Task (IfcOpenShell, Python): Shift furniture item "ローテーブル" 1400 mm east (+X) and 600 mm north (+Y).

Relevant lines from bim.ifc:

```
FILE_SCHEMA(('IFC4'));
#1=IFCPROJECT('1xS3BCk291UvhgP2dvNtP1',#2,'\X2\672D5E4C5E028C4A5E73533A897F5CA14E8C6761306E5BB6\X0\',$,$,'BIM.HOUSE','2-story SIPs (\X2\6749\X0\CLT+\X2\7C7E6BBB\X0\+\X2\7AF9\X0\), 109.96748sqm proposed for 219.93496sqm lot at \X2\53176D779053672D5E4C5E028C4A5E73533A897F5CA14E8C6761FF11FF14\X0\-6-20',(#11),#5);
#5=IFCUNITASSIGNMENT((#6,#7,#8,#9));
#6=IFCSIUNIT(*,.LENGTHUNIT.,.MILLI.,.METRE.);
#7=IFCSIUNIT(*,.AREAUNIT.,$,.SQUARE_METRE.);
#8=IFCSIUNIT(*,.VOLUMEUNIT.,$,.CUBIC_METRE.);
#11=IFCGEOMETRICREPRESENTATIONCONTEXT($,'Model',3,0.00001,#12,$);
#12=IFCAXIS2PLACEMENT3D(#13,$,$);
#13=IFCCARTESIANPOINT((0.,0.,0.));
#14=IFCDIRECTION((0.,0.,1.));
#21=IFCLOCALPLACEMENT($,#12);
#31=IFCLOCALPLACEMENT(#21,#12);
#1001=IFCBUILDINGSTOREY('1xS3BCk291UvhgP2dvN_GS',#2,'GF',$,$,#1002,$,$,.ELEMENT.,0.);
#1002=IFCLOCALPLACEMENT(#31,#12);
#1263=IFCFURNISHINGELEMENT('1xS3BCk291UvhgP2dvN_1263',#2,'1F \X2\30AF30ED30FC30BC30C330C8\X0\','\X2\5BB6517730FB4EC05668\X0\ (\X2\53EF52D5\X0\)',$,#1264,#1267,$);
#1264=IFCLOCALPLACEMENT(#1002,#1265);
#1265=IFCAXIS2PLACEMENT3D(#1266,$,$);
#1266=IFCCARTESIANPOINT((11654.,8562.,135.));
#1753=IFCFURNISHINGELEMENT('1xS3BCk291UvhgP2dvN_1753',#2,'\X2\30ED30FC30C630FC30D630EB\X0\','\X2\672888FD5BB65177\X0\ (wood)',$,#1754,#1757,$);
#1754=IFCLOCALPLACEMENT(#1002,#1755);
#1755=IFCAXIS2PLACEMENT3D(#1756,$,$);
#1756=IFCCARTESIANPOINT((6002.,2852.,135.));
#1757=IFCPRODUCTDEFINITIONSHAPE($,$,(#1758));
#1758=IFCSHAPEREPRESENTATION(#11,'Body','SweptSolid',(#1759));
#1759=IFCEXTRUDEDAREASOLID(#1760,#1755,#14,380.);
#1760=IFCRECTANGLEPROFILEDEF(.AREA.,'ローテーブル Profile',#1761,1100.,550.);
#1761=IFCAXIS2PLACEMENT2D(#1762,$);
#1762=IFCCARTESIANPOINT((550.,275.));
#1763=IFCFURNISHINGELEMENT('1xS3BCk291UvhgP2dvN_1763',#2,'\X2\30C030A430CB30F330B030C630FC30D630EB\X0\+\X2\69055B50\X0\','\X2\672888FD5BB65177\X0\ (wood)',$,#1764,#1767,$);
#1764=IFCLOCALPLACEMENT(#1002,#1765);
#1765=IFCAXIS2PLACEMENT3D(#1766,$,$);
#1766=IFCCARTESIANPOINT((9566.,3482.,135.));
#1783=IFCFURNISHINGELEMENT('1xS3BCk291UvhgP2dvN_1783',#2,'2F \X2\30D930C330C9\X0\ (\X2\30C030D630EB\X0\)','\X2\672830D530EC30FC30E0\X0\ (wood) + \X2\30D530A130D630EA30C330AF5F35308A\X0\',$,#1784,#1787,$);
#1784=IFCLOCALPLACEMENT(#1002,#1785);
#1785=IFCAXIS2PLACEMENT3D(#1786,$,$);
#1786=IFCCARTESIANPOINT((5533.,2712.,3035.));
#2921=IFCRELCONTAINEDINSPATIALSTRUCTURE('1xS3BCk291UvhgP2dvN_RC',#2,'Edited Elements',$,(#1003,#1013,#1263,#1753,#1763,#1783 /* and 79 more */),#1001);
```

```python
import ifcopenshell
import ifcopenshell.api.geometry
import ifcopenshell.util.placement

model = ifcopenshell.open("bim.ifc")

item = model.by_id(1753)
matrix = ifcopenshell.util.placement.get_local_placement(item.ObjectPlacement)
matrix[0, 3] += 1400.0
matrix[1, 3] += 600.0
ifcopenshell.api.geometry.edit_object_placement(model, product=item, matrix=matrix, is_si=False)

print(ifcopenshell.util.placement.get_local_placement(item.ObjectPlacement).round(3) + 0.0)

model.write("bim_updated.ifc")
```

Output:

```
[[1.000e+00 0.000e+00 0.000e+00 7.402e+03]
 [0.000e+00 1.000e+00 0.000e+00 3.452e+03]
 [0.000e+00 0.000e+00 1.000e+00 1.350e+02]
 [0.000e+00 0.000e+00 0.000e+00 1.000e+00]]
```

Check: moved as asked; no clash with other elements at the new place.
